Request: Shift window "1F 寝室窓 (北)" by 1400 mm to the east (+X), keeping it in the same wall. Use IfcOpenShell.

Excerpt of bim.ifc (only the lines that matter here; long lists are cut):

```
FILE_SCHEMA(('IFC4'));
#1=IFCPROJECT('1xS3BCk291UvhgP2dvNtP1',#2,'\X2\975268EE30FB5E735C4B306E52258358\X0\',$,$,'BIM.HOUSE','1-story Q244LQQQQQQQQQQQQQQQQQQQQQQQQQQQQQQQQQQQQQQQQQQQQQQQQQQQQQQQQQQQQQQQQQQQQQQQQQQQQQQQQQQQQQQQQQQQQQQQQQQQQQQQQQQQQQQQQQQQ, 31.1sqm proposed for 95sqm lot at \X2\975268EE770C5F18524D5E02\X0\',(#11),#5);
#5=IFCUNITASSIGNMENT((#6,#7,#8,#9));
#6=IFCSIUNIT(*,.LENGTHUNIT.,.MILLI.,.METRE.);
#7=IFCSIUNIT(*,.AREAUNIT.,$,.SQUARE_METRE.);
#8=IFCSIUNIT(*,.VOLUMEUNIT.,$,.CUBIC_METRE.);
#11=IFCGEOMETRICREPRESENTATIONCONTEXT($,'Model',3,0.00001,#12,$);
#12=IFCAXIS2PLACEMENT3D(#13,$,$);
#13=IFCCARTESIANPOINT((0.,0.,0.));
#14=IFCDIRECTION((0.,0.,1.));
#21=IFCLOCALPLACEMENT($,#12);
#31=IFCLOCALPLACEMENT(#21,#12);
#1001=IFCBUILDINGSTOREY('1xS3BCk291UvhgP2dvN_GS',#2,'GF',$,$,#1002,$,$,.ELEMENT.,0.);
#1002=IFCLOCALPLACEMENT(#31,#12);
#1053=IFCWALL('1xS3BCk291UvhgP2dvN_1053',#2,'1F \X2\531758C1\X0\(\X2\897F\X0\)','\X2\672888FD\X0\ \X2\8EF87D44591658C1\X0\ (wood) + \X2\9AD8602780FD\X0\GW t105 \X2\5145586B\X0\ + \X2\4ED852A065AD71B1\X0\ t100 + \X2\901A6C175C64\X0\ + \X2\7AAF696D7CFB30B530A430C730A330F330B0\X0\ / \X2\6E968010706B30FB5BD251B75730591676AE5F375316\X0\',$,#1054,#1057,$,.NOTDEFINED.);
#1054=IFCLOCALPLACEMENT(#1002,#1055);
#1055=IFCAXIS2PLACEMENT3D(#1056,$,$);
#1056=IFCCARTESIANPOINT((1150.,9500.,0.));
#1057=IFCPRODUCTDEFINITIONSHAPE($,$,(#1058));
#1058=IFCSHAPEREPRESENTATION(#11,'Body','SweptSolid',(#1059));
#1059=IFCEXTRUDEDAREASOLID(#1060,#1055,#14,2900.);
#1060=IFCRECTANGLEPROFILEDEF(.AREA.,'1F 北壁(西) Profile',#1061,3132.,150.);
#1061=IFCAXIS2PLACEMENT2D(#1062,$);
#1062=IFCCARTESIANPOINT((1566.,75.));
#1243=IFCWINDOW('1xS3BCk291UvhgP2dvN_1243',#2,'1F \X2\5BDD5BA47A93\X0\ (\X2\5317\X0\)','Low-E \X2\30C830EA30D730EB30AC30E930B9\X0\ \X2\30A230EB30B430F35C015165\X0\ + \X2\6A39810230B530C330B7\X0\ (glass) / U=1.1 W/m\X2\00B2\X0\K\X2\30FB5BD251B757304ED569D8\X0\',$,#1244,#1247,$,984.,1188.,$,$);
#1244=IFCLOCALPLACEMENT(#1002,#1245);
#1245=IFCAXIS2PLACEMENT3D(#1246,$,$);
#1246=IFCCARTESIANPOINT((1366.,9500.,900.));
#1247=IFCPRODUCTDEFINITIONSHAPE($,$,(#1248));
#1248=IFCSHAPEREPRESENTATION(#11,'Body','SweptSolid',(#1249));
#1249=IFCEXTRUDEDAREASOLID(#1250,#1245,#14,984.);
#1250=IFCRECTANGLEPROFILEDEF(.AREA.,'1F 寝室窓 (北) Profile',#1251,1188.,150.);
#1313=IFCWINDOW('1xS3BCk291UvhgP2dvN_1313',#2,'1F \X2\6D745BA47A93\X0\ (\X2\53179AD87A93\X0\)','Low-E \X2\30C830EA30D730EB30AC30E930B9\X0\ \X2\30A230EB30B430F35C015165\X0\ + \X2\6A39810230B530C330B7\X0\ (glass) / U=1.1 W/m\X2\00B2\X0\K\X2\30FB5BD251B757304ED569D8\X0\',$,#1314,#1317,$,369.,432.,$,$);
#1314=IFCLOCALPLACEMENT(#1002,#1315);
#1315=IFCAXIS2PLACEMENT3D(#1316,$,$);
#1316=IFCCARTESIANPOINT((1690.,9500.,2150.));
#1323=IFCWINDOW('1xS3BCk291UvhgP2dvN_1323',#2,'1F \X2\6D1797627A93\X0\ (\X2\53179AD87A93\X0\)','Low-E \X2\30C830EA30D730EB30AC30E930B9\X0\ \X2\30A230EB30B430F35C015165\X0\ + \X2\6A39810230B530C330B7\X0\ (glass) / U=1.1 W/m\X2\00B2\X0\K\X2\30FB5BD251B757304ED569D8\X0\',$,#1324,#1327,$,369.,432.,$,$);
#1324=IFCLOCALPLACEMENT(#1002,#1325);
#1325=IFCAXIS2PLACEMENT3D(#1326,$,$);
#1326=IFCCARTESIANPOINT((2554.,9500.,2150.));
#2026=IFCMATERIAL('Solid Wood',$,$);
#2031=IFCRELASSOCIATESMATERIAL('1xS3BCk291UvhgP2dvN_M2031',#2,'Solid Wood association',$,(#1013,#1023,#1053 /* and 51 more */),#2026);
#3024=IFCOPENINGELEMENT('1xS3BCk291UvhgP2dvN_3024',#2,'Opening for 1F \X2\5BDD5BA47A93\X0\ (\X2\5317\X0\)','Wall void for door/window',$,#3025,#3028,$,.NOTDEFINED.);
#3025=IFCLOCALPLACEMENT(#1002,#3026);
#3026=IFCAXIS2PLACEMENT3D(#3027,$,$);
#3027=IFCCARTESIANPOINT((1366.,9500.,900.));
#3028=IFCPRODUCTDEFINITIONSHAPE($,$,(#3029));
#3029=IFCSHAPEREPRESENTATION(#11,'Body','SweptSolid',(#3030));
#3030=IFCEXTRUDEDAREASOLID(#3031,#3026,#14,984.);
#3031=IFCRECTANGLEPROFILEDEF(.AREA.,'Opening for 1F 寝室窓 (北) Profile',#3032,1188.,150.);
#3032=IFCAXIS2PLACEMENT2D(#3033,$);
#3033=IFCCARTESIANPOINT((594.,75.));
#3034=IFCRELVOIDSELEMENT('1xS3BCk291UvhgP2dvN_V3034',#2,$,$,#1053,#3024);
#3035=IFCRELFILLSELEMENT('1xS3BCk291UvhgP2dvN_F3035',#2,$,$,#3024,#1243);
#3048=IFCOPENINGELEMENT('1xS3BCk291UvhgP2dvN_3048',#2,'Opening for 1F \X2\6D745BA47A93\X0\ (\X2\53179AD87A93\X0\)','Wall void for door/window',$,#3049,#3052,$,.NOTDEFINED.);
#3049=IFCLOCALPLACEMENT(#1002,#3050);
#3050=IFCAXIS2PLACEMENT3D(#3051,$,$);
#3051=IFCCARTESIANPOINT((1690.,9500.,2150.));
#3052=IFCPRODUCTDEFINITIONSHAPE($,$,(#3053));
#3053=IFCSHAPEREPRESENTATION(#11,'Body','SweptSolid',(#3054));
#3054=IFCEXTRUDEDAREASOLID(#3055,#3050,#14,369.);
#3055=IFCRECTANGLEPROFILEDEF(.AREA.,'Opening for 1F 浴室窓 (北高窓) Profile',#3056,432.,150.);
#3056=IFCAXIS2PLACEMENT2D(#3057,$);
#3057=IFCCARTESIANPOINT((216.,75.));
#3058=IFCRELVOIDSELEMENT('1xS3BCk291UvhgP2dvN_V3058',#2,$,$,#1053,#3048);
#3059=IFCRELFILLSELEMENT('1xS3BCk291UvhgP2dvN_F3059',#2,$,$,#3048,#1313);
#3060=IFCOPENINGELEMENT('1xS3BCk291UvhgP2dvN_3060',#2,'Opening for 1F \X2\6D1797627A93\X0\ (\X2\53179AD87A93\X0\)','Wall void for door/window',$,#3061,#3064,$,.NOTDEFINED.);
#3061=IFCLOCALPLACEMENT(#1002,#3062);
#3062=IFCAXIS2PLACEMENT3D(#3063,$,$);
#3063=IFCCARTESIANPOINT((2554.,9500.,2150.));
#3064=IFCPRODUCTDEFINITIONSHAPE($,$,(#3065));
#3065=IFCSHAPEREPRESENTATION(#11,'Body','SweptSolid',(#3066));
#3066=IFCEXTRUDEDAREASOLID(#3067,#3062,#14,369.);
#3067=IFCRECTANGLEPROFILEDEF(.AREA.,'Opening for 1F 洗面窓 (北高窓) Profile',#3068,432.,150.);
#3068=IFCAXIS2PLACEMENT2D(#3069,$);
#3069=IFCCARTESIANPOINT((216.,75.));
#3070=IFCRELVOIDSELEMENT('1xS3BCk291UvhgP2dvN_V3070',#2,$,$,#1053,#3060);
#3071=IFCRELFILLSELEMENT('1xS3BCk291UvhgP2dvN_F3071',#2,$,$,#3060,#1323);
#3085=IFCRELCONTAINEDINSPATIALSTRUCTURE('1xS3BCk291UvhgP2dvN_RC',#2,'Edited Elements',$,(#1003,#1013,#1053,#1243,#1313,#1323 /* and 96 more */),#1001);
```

```python
import ifcopenshell
import ifcopenshell.api.geometry
import ifcopenshell.util.placement

model = ifcopenshell.open("bim.ifc")

window = model.by_guid("1xS3BCk291UvhgP2dvN_1243")
opening = window.FillsVoids[0].RelatingOpeningElement
wall = opening.VoidsElements[0].RelatingBuildingElement

wall_matrix = ifcopenshell.util.placement.get_local_placement(wall.ObjectPlacement)
shift = wall_matrix[:3, 0] * 1400.0
before = ifcopenshell.util.placement.get_local_placement(window.ObjectPlacement)[:3, 3].copy()

# The window is not placed relative to its opening, so move both.
for product in (opening, window):
    matrix = ifcopenshell.util.placement.get_local_placement(product.ObjectPlacement)
    matrix[:3, 3] += shift
    ifcopenshell.api.geometry.edit_object_placement(model, product=product, matrix=matrix, is_si=False)

after = ifcopenshell.util.placement.get_local_placement(window.ObjectPlacement)[:3, 3]
print("window moved by", (after - before).round(3) + 0.0)

model.write("bim_v2.ifc")
```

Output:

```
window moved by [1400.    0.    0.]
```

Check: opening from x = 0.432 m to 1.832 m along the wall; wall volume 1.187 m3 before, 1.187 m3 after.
